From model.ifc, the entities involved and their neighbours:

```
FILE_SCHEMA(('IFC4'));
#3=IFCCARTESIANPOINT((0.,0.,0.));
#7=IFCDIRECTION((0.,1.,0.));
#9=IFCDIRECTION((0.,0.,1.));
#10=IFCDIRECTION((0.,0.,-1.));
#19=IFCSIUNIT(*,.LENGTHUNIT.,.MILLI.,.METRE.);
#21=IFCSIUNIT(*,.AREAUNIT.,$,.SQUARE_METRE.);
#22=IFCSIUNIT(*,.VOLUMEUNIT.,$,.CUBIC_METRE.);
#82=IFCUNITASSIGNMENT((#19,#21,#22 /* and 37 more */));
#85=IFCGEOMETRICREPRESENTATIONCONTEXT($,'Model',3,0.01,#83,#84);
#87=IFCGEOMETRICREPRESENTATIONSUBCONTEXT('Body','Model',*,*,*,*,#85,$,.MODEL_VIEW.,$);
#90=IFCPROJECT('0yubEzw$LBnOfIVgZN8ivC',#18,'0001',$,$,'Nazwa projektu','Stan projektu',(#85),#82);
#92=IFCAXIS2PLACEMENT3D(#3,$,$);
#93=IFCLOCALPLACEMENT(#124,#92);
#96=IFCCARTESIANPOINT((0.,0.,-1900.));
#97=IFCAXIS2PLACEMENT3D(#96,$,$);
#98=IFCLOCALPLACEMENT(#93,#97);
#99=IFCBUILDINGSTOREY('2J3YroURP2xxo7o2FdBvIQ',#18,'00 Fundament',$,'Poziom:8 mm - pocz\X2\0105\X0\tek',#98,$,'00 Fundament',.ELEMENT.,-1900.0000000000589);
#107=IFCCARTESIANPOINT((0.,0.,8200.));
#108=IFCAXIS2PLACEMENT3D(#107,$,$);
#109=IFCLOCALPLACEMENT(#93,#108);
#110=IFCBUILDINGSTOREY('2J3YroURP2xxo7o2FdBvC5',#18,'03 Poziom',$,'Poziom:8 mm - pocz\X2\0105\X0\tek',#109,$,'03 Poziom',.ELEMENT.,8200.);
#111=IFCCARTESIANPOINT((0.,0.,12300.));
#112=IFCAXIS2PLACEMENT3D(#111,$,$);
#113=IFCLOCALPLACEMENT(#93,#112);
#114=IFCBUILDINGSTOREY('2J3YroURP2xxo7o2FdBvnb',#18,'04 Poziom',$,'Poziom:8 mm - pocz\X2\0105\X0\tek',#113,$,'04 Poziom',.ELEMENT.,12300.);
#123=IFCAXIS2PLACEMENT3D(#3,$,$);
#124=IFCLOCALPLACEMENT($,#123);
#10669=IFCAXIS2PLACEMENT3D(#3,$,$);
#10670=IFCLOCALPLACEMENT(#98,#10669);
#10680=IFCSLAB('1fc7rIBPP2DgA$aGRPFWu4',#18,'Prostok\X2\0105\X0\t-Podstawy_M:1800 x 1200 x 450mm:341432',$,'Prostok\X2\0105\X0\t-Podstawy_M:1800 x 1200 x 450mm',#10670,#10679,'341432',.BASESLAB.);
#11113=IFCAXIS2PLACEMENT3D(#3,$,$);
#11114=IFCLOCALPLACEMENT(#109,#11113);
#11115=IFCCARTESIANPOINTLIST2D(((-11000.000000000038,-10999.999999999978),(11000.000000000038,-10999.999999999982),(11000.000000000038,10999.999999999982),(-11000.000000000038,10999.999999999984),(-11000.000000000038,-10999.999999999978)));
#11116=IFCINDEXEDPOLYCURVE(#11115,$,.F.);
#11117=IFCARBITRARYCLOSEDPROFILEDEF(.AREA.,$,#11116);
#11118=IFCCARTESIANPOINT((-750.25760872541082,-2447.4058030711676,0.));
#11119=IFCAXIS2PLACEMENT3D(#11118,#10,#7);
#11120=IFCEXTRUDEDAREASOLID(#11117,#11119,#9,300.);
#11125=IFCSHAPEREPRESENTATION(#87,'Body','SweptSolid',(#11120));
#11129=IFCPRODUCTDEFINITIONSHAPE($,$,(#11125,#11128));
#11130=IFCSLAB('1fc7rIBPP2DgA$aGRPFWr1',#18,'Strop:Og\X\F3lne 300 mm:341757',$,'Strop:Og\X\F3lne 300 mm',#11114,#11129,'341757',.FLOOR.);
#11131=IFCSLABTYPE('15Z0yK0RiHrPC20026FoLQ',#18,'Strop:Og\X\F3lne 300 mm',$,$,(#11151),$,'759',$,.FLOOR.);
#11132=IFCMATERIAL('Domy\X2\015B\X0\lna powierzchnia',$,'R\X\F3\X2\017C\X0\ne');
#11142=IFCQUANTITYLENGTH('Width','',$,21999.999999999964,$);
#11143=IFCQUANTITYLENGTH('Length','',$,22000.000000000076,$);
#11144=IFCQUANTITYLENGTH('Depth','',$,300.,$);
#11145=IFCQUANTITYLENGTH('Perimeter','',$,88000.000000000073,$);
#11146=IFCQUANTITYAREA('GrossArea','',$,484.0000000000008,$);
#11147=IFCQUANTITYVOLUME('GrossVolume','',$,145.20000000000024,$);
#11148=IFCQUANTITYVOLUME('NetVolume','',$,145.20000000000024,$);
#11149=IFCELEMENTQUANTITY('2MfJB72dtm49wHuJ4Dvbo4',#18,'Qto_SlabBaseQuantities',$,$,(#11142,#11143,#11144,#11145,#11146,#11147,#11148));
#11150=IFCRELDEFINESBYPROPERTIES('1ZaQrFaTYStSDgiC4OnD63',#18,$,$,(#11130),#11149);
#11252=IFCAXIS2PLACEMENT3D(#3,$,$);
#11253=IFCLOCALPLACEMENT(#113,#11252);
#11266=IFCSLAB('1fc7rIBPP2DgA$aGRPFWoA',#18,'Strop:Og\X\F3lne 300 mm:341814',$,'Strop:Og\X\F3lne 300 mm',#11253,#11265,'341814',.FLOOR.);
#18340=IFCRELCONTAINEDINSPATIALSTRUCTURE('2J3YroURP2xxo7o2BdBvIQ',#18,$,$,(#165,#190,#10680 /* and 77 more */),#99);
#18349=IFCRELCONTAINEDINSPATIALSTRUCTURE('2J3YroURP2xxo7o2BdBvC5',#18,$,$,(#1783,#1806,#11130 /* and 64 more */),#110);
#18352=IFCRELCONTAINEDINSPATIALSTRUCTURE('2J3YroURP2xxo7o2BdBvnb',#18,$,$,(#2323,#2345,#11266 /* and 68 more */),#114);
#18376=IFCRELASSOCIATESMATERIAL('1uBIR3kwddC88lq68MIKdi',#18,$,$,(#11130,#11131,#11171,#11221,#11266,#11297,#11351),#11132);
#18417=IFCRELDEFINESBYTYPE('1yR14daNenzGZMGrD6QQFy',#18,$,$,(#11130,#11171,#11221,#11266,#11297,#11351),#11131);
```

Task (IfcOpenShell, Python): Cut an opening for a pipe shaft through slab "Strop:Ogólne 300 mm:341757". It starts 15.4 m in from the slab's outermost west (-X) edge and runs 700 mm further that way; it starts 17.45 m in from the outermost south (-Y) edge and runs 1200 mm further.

```python
import numpy as np
import ifcopenshell
import ifcopenshell.api.feature
import ifcopenshell.api.geometry
import ifcopenshell.api.pset
import ifcopenshell.api.root
import ifcopenshell.geom
import ifcopenshell.util.element
import ifcopenshell.util.placement
import ifcopenshell.util.representation
import ifcopenshell.util.shape
import ifcopenshell.util.unit

model = ifcopenshell.open("model.ifc")
unit_scale = ifcopenshell.util.unit.calculate_unit_scale(model)
volume_scale = ifcopenshell.util.unit.calculate_unit_scale(model, "VOLUMEUNIT")
settings = ifcopenshell.geom.settings()


def volume(element):
    """Net volume in cubic metres, openings subtracted."""
    shape = ifcopenshell.geom.create_shape(settings, element)
    return ifcopenshell.util.shape.get_volume(shape.geometry)


slab = model.by_guid("1fc7rIBPP2DgA$aGRPFWr1")
before = volume(slab)

# Extent in the slab's own axes, in metres. The edges named are its -X and -Y sides.
slab_shape = ifcopenshell.geom.create_shape(settings, slab)
vertices = ifcopenshell.util.shape.get_vertices(slab_shape.geometry)
x_min, y_min, bottom = vertices.min(axis=0)
top = vertices[:, 2].max()

opening = ifcopenshell.api.root.create_entity(model, ifc_class="IfcOpeningElement", name="Pipe shaft opening", predefined_type="OPENING")
context = ifcopenshell.util.representation.get_context(model, "Model", "Body", "MODEL_VIEW")
width, depth = 0.7, 1.2
outline = [(0.0, 0.0), (width, 0.0), (width, depth), (0.0, depth), (0.0, 0.0)]
# Overshoot both faces by 50 mm so the cut is clean.
shape = ifcopenshell.api.geometry.add_slab_representation(
    model, context=context, depth=top - bottom + 0.1, polyline=outline
)
ifcopenshell.api.geometry.assign_representation(model, product=opening, representation=shape)

matrix = ifcopenshell.util.placement.get_local_placement(slab.ObjectPlacement)
matrix[:, 3] = matrix @ np.append(np.array([x_min + 15.4, y_min + 17.45, bottom - 0.05]) / unit_scale, 1.0)
ifcopenshell.api.geometry.edit_object_placement(model, product=opening, matrix=matrix, is_si=False)
ifcopenshell.api.feature.add_feature(model, feature=opening, element=slab)

after = volume(slab)

# Update the slab's stored quantities.
qto = model.by_id(ifcopenshell.util.element.get_pset(slab, "Qto_SlabBaseQuantities", should_inherit=False)["id"])
ifcopenshell.api.pset.edit_qto(model, qto=qto, properties={"NetVolume": after / volume_scale})

print(f"slab volume {before:.3f} -> {after:.3f} m3")

model.write("model_edited.ifc")
```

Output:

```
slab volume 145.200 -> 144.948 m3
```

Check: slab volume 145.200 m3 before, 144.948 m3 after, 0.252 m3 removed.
